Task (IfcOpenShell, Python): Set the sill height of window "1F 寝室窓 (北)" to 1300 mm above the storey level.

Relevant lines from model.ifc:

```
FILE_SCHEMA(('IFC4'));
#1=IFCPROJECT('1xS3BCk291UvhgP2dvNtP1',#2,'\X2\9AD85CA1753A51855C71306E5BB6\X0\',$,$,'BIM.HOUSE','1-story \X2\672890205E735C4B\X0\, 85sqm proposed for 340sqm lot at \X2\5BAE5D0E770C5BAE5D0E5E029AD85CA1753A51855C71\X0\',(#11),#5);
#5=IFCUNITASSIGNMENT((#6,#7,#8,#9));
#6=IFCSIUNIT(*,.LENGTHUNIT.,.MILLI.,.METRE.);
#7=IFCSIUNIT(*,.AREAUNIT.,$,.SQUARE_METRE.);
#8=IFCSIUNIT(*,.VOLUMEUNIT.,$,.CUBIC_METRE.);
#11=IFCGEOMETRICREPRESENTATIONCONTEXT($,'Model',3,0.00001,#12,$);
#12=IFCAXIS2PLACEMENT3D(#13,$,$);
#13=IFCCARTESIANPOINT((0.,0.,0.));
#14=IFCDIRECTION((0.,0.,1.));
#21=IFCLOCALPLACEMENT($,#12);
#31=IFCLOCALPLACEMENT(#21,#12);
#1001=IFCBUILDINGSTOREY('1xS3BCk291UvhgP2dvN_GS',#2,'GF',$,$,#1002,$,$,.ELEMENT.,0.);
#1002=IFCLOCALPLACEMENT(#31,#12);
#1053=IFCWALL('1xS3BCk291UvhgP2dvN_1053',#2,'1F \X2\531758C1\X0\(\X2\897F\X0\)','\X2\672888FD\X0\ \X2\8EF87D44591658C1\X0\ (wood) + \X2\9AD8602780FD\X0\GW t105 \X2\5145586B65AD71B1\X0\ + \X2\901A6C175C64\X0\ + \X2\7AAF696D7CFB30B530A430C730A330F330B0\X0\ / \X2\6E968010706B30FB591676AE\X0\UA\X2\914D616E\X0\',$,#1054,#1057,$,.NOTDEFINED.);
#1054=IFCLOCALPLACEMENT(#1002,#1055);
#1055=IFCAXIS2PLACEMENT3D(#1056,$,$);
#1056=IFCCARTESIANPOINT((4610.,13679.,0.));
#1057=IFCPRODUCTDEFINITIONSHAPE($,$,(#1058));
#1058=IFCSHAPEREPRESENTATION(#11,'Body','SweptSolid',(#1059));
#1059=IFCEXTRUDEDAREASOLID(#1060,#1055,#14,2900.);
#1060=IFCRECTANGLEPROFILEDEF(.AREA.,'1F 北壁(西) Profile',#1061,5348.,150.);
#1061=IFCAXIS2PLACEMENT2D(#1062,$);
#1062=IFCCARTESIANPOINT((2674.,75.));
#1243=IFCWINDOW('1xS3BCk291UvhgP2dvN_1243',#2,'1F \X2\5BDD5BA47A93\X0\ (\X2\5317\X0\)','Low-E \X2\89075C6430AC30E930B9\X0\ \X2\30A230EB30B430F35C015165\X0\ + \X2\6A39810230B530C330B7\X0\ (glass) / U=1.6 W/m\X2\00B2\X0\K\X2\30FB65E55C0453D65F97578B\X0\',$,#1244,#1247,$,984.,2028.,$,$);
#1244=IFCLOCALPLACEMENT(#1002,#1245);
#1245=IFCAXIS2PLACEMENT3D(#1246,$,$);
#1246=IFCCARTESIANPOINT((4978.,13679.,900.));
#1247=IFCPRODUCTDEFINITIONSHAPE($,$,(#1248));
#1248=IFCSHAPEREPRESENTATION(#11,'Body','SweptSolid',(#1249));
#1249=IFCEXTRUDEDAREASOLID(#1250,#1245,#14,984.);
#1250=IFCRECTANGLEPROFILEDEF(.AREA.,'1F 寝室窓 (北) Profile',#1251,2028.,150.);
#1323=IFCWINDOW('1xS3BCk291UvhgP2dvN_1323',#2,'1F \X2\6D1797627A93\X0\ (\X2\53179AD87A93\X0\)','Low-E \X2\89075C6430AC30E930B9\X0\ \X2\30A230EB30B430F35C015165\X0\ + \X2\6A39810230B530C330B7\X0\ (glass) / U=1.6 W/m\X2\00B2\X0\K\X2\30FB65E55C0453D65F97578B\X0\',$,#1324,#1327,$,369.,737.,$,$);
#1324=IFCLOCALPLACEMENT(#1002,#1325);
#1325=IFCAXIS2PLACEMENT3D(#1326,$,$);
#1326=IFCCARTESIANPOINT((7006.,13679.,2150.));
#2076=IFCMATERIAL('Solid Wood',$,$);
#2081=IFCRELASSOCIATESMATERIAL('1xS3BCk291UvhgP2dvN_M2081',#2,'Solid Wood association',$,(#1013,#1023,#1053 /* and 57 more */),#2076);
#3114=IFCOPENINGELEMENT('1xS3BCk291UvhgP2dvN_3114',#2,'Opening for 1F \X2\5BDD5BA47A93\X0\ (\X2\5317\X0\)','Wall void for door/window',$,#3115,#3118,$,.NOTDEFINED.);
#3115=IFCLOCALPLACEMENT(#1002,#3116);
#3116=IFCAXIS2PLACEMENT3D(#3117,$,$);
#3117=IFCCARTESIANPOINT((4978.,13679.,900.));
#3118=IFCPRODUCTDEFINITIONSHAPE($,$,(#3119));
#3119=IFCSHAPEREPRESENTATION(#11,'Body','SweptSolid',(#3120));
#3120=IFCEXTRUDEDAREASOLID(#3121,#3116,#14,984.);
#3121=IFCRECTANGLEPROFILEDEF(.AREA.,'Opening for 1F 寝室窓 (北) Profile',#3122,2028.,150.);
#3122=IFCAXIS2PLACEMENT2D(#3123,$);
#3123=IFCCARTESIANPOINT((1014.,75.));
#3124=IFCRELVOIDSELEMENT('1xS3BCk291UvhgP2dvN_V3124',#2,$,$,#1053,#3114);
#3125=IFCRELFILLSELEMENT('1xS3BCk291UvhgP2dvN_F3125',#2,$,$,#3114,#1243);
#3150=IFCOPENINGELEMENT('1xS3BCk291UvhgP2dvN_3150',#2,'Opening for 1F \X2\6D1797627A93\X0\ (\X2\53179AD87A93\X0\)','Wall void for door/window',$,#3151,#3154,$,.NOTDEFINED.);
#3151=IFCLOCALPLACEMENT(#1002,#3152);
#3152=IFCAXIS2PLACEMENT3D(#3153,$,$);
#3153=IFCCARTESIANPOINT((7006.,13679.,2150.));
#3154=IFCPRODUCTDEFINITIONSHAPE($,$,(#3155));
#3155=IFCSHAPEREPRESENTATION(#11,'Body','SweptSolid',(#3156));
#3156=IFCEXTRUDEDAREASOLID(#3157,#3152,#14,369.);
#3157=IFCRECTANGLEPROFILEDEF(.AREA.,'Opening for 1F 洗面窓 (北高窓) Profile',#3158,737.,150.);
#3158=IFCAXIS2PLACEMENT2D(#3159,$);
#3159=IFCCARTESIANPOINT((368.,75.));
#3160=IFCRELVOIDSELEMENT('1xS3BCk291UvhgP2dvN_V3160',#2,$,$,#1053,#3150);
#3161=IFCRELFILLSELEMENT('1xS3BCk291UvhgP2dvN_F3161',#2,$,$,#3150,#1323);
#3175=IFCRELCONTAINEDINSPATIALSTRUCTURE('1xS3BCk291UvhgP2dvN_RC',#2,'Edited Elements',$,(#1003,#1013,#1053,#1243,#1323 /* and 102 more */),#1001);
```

```python
import numpy as np
import ifcopenshell
import ifcopenshell.api.geometry
import ifcopenshell.geom
import ifcopenshell.util.element
import ifcopenshell.util.placement
import ifcopenshell.util.shape
import ifcopenshell.util.unit

model = ifcopenshell.open("model.ifc")
unit_scale = ifcopenshell.util.unit.calculate_unit_scale(model)

window = model.by_guid("1xS3BCk291UvhgP2dvN_1243")
opening = window.FillsVoids[0].RelatingOpeningElement
storey = ifcopenshell.util.element.get_container(window, ifc_class="IfcBuildingStorey")
level = ifcopenshell.util.placement.get_local_placement(storey.ObjectPlacement)[2, 3]

# The opening's origin need not be at the sill, so measure its lowest point.
shape = ifcopenshell.geom.create_shape(ifcopenshell.geom.settings(), opening)
bottom = ifcopenshell.util.shape.get_shape_bottom_elevation(shape, shape.geometry) / unit_scale
dz = level + 1.3 / unit_scale - bottom

shift = np.array([0.0, 0.0, dz])
# The window is not placed relative to its opening, so move both.
for product in (opening, window):
    matrix = ifcopenshell.util.placement.get_local_placement(product.ObjectPlacement)
    matrix[:3, 3] += shift
    ifcopenshell.api.geometry.edit_object_placement(model, product=product, matrix=matrix, is_si=False)

print(f"moved by {dz * unit_scale:+.3f} m")

model.write("model_v2.ifc")
```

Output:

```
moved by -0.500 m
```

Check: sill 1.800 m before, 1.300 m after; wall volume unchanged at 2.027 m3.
